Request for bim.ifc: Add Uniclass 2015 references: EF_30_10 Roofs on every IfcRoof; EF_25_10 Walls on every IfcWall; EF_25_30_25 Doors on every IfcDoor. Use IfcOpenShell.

First a look at what the model holds.

```python
import ifcopenshell

model = ifcopenshell.open("bim.ifc")
print(model.schema)
print("classifications:", [c.Name for c in model.by_type("IfcClassification")])
for ifc_class in ("IfcDoor", "IfcRoof", "IfcStair", "IfcWall", "IfcWindow"):
    print(ifc_class, len(model.by_type(ifc_class)))
```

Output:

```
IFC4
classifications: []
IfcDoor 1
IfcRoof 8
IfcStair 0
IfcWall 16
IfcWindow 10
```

```python
import ifcopenshell
import ifcopenshell.api.classification

model = ifcopenshell.open("bim.ifc")

system = ifcopenshell.api.classification.add_classification(model, classification="Uniclass 2015")

codes = {
    "IfcRoof": ("EF_30_10", "Roofs"),
    "IfcWall": ("EF_25_10", "Walls"),
    "IfcDoor": ("EF_25_30_25", "Doors"),
}
for ifc_class, (code, name) in codes.items():
    products = model.by_type(ifc_class)
    ifcopenshell.api.classification.add_reference(
        model, products=products, classification=system, identification=code, name=name
    )
    print(code, len(products))

model.write("bim_updated.ifc")
```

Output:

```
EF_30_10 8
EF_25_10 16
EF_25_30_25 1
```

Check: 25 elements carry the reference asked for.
